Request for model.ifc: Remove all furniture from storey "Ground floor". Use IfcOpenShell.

First a look at what the model holds.

```python
import ifcopenshell
import ifcopenshell.util.element

model = ifcopenshell.open("model.ifc")
print(model.schema)
storey = next(s for s in model.by_type("IfcBuildingStorey") if s.Name == "Ground floor")
furniture = [e for e in ifcopenshell.util.element.get_decomposition(storey) if e.is_a("IfcFurnishingElement")]
seen = {}
for e in furniture:
    element_type = ifcopenshell.util.element.get_type(e)
    name = element_type.Name if element_type not in (None, e) else None
    seen[name] = seen.get(name, 0) + 1
for name, count in sorted(seen.items(), key=str):
    print(count, "x", name)
```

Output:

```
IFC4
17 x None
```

```python
import ifcopenshell
import ifcopenshell.api.root
import ifcopenshell.util.element

model = ifcopenshell.open("model.ifc")

storey = next(s for s in model.by_type("IfcBuildingStorey") if s.Name == "Ground floor")
furniture = [e for e in ifcopenshell.util.element.get_decomposition(storey) if e.is_a("IfcFurnishingElement")]

for e in furniture:
    ifcopenshell.api.root.remove_product(model, product=e)
print(len(furniture), "removed")

model.write("model_updated.ifc")
```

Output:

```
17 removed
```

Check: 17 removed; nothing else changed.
